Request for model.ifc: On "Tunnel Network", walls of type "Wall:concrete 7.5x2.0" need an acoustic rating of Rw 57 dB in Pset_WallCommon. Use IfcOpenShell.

First a look at what the model holds.

```python
import ifcopenshell
import ifcopenshell.util.element

model = ifcopenshell.open("model.ifc")
print(model.schema)
storey = next(s for s in model.by_type("IfcBuildingStorey") if s.Name == "Tunnel Network")
walls = [e for e in ifcopenshell.util.element.get_decomposition(storey) if e.is_a("IfcWall")]
seen = {}
for e in walls:
    element_type = ifcopenshell.util.element.get_type(e)
    key = (element_type.Name if element_type != e and element_type else None, ifcopenshell.util.element.get_pset(e, "Pset_WallCommon", "AcousticRating"))
    seen[key] = seen.get(key, 0) + 1
for (name, value), count in sorted(seen.items(), key=str):
    print(count, "x", name, "|", value)
```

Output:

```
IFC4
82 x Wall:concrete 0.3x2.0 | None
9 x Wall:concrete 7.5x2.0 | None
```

```python
import ifcopenshell
import ifcopenshell.api.pset
import ifcopenshell.util.element

model = ifcopenshell.open("model.ifc")

storey = next(s for s in model.by_type("IfcBuildingStorey") if s.Name == "Tunnel Network")
walls = [e for e in ifcopenshell.util.element.get_decomposition(storey) if e.is_a("IfcWall")]

count = 0
for e in walls:
    element_type = ifcopenshell.util.element.get_type(e)
    if element_type in (None, e) or element_type.Name != "Wall:concrete 7.5x2.0":
        continue
    # add_pset returns the element's existing set when there is one.
    pset = ifcopenshell.api.pset.add_pset(model, product=e, name="Pset_WallCommon")
    ifcopenshell.api.pset.edit_pset(model, pset=pset, properties={"AcousticRating": "Rw 57 dB"})
    count += 1

print(count, "walls updated")

model.write("model_rev.ifc")
```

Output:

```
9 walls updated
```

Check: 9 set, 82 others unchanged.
